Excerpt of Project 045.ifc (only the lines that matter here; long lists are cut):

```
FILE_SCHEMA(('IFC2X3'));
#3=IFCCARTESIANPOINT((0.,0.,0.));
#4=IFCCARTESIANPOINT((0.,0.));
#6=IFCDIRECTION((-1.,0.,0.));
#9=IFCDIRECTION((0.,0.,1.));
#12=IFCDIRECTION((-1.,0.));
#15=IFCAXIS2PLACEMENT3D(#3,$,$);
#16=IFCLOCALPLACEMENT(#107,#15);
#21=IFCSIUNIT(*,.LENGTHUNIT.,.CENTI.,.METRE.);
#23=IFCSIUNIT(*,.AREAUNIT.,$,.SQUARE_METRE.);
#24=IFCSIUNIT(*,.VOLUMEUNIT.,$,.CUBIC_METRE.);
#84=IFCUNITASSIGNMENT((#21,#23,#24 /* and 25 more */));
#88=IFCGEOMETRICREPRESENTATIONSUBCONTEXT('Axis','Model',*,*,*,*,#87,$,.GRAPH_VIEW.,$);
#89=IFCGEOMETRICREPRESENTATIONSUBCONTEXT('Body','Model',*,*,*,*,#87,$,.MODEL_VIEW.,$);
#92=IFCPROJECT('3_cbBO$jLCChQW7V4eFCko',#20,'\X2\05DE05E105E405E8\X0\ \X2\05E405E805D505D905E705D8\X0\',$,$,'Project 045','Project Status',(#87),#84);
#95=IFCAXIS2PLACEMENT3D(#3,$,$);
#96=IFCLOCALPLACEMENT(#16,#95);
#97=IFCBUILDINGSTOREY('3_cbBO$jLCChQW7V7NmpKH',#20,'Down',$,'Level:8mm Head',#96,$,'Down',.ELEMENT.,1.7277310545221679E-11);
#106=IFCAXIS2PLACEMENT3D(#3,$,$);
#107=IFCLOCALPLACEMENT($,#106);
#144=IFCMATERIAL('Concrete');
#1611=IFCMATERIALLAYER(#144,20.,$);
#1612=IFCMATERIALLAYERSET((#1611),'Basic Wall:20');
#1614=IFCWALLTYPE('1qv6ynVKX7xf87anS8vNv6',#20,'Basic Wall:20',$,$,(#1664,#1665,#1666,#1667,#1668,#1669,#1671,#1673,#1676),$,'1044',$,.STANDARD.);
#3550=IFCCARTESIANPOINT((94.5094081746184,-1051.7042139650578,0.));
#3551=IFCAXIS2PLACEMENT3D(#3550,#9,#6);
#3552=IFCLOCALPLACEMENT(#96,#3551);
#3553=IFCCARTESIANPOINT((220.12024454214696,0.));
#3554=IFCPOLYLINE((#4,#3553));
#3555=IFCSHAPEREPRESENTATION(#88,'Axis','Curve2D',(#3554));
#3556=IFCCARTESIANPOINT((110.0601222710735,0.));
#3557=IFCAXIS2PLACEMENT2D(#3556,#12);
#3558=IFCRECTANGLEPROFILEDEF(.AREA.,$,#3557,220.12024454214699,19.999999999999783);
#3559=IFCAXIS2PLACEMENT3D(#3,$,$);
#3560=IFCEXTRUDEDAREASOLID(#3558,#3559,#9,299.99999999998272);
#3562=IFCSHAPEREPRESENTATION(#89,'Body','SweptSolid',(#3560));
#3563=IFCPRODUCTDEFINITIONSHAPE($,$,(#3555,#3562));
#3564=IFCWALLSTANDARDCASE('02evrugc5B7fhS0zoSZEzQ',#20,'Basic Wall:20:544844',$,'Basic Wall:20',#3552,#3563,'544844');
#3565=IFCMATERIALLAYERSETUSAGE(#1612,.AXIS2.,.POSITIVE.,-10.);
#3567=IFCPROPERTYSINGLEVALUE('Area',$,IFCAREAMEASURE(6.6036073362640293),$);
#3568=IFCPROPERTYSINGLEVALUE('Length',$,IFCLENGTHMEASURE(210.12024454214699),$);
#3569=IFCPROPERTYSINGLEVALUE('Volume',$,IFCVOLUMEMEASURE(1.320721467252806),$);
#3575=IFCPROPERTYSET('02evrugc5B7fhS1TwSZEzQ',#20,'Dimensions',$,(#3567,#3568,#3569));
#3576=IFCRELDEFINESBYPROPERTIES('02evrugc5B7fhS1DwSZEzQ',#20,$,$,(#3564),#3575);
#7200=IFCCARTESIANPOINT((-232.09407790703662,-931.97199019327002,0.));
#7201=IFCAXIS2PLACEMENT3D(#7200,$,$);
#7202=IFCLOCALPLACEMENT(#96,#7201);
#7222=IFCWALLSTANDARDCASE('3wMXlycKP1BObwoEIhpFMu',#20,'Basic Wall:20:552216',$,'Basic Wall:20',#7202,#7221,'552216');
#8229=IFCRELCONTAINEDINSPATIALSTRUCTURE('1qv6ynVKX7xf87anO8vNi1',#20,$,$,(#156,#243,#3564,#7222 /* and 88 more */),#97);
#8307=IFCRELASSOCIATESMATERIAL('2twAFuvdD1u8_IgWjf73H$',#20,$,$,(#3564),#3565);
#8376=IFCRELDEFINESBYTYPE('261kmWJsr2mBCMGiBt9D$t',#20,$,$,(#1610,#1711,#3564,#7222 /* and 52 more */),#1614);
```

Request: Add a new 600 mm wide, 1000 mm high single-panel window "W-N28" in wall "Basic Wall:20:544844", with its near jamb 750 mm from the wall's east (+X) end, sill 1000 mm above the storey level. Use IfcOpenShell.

```python
import numpy as np
import ifcopenshell
import ifcopenshell.api.feature
import ifcopenshell.api.geometry
import ifcopenshell.api.pset
import ifcopenshell.api.root
import ifcopenshell.api.spatial
import ifcopenshell.api.type
import ifcopenshell.geom
import ifcopenshell.util.element
import ifcopenshell.util.placement
import ifcopenshell.util.representation
import ifcopenshell.util.shape
import ifcopenshell.util.unit

model = ifcopenshell.open("Project 045.ifc")
unit_scale = ifcopenshell.util.unit.calculate_unit_scale(model)
area_scale = ifcopenshell.util.unit.calculate_unit_scale(model, "AREAUNIT")
volume_scale = ifcopenshell.util.unit.calculate_unit_scale(model, "VOLUMEUNIT")
settings = ifcopenshell.geom.settings()


def volume(element):
    """Net volume in cubic metres, openings subtracted."""
    shape = ifcopenshell.geom.create_shape(settings, element)
    return ifcopenshell.util.shape.get_volume(shape.geometry)


wall = model.by_guid("02evrugc5B7fhS0zoSZEzQ")
storey = ifcopenshell.util.element.get_container(wall, ifc_class="IfcBuildingStorey")
context = ifcopenshell.util.representation.get_context(model, "Model", "Body", "MODEL_VIEW")
before = volume(wall)

width, height, from_end, sill = 0.6, 1, 0.75, 1  # metres

# The wall runs along its own X axis, and the end named is its -X end.
wall_shape = ifcopenshell.geom.create_shape(settings, wall)
x, y, z = ifcopenshell.util.shape.get_vertices(wall_shape.geometry).T
start = x.min() + from_end
face, thickness = float(y.min()), float(y.max() - y.min())
wall_matrix = ifcopenshell.util.placement.get_local_placement(wall.ObjectPlacement)
level = ifcopenshell.util.placement.get_local_placement(storey.ObjectPlacement)[2, 3]


def in_wall(x, y):
    """Placement at x, y metres in the wall's axes, at sill height."""
    matrix = wall_matrix.copy()
    matrix[:, 3] = wall_matrix @ np.array([x / unit_scale, y / unit_scale, 0.0, 1.0])
    matrix[2, 3] = level + sill / unit_scale
    return matrix


# Opening: a box that overshoots both wall faces by 50 mm.
opening = ifcopenshell.api.root.create_entity(model, ifc_class="IfcOpeningElement")
box = ifcopenshell.api.geometry.add_wall_representation(
    model, context=context, length=width, height=height, thickness=thickness + 0.1
)
ifcopenshell.api.geometry.assign_representation(model, product=opening, representation=box)
ifcopenshell.api.geometry.edit_object_placement(model, product=opening, matrix=in_wall(start, face - 0.05), is_si=False)
ifcopenshell.api.feature.add_feature(model, feature=opening, element=wall)

window = ifcopenshell.api.root.create_entity(model, ifc_class="IfcWindow", name="W-N28")
window.OverallWidth, window.OverallHeight = width / unit_scale, height / unit_scale
body = ifcopenshell.api.geometry.add_window_representation(
    model,
    context=context,
    overall_width=window.OverallWidth,
    overall_height=window.OverallHeight,
    partition_type="SINGLE_PANEL",
)
ifcopenshell.api.geometry.assign_representation(model, product=window, representation=body)
ifcopenshell.api.spatial.assign_container(model, products=[window], relating_structure=storey)
fills = ifcopenshell.api.feature.add_filling(model, opening=opening, element=window)
fills.OwnerHistory = window.OwnerHistory  # required in IFC2X3

# IFC2X3 keeps the operation on the window style.
style = ifcopenshell.api.root.create_entity(model, ifc_class="IfcWindowStyle", name="W-N28")
style.OperationType, style.ConstructionType = "SINGLE_PANEL", "NOTDEFINED"
style.ParameterTakesPrecedence = style.Sizeable = False
ifcopenshell.api.type.assign_type(model, related_objects=[window], relating_type=style)

# Centre the window in the wall's thickness.
ifcopenshell.api.geometry.edit_object_placement(model, product=window, matrix=in_wall(start, face), is_si=False)
window_shape = ifcopenshell.geom.create_shape(settings, window)
depth = ifcopenshell.util.shape.get_vertices(window_shape.geometry)[:, 1]
offset = face + thickness / 2 - (depth.min() + depth.max()) / 2
ifcopenshell.api.geometry.edit_object_placement(model, product=window, matrix=in_wall(start, offset), is_si=False)

after = volume(wall)

# Update the wall's stored quantities.
pset = model.by_id(ifcopenshell.util.element.get_pset(wall, "Dimensions", should_inherit=False)["id"])
ifcopenshell.api.pset.edit_pset(model, pset=pset, properties={
    "Area": model.create_entity("IfcAreaMeasure", after / thickness / area_scale),
    "Volume": model.create_entity("IfcVolumeMeasure", after / volume_scale),
})

print(f"wall volume {before:.3f} -> {after:.3f} m3")

model.write("Project 045_updated.ifc")
```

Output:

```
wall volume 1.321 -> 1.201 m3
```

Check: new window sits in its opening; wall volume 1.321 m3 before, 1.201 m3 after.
